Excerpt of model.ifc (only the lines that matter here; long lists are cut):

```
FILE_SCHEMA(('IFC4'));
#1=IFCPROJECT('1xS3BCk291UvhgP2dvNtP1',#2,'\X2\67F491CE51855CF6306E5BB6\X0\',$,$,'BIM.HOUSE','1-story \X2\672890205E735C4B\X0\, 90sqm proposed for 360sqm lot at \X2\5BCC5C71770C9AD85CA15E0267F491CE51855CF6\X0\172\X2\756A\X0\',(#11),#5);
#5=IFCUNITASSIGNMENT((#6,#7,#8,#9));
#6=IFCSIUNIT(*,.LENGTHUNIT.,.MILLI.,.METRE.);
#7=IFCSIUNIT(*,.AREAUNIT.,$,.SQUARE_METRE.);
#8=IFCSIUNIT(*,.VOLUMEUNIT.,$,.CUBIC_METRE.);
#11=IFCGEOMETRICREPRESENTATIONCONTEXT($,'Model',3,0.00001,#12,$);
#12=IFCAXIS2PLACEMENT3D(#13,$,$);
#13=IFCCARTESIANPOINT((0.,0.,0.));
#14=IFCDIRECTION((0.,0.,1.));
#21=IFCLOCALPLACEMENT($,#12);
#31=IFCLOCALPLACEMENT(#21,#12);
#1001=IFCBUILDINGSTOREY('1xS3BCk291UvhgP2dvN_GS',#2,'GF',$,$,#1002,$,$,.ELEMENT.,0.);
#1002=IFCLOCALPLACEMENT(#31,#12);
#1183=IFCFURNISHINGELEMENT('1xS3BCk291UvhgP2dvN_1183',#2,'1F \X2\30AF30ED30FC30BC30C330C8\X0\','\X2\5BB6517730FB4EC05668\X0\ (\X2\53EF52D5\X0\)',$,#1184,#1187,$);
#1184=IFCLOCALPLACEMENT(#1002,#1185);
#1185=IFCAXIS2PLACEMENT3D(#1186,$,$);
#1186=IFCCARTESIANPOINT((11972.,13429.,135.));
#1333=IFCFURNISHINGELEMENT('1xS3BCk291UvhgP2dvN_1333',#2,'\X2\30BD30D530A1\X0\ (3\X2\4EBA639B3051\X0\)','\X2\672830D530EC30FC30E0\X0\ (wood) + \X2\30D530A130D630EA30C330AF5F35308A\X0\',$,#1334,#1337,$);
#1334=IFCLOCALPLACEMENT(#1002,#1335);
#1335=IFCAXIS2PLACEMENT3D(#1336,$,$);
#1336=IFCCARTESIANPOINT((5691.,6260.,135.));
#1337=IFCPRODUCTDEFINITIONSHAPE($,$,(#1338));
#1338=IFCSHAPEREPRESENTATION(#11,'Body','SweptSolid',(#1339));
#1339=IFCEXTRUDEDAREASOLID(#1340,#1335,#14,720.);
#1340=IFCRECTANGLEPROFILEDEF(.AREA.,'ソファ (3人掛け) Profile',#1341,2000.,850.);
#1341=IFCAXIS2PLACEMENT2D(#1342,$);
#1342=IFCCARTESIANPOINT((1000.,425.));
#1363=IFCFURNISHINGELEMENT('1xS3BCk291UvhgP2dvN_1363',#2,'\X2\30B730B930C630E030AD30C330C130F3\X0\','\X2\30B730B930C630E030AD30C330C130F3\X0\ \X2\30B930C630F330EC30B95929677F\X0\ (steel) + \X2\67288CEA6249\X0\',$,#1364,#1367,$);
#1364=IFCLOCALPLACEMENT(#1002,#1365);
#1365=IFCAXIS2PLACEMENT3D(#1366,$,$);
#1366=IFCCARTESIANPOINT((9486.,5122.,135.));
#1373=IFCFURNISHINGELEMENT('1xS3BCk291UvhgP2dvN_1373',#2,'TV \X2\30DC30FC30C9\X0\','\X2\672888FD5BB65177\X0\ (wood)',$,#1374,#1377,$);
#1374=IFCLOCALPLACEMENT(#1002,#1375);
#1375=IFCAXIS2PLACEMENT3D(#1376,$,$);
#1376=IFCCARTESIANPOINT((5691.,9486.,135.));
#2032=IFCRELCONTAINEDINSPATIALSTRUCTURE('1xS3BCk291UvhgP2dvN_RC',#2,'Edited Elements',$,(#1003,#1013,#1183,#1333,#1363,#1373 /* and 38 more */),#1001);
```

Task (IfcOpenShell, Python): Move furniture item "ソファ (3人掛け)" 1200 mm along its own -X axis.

```python
import ifcopenshell
import ifcopenshell.api.geometry
import ifcopenshell.util.placement
import ifcopenshell.util.unit

model = ifcopenshell.open("model.ifc")
unit_scale = ifcopenshell.util.unit.calculate_unit_scale(model)

item = model.by_id(1333)
matrix = ifcopenshell.util.placement.get_local_placement(item.ObjectPlacement)
matrix[:3, 3] -= matrix[:3, 0] * 1.2 / unit_scale
ifcopenshell.api.geometry.edit_object_placement(model, product=item, matrix=matrix, is_si=False)

print(ifcopenshell.util.placement.get_local_placement(item.ObjectPlacement).round(3) + 0.0)

model.write("model_edited.ifc")
```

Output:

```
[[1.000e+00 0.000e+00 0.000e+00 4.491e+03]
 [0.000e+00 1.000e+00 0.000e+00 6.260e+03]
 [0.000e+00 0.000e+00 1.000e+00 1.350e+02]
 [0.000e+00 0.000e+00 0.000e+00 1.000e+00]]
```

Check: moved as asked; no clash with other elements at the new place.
